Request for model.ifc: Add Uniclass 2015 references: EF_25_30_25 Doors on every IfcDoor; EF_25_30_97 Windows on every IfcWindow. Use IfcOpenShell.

First a look at what the model holds.

```python
import ifcopenshell

model = ifcopenshell.open("model.ifc")
print(model.schema)
print("classifications:", [c.Name for c in model.by_type("IfcClassification")])
for ifc_class in ("IfcDoor", "IfcRoof", "IfcStair", "IfcWall", "IfcWindow"):
    print(ifc_class, len(model.by_type(ifc_class)))
```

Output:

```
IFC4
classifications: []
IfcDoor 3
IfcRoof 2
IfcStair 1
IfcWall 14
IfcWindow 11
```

```python
import ifcopenshell
import ifcopenshell.api.classification

model = ifcopenshell.open("model.ifc")

system = ifcopenshell.api.classification.add_classification(model, classification="Uniclass 2015")

codes = {
    "IfcDoor": ("EF_25_30_25", "Doors"),
    "IfcWindow": ("EF_25_30_97", "Windows"),
}
for ifc_class, (code, name) in codes.items():
    products = model.by_type(ifc_class)
    ifcopenshell.api.classification.add_reference(
        model, products=products, classification=system, identification=code, name=name
    )
    print(code, len(products))

model.write("model_rev.ifc")
```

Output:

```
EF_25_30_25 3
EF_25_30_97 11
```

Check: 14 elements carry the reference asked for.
